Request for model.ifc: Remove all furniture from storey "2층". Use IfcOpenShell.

First a look at what the model holds.

```python
import ifcopenshell
import ifcopenshell.util.element

model = ifcopenshell.open("model.ifc")
print(model.schema)
storey = next(s for s in model.by_type("IfcBuildingStorey") if s.Name == "2층")
furniture = [e for e in ifcopenshell.util.element.get_decomposition(storey) if e.is_a("IfcFurnishingElement")]
seen = {}
for e in furniture:
    element_type = ifcopenshell.util.element.get_type(e)
    name = element_type.Name if element_type not in (None, e) else None
    seen[name] = seen.get(name, 0) + 1
for name, count in sorted(seen.items(), key=str):
    print(count, "x", name)
```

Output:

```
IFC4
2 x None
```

```python
import ifcopenshell
import ifcopenshell.api.root
import ifcopenshell.util.element

model = ifcopenshell.open("model.ifc")

storey = next(s for s in model.by_type("IfcBuildingStorey") if s.Name == "2층")
furniture = [e for e in ifcopenshell.util.element.get_decomposition(storey) if e.is_a("IfcFurnishingElement")]

for e in furniture:
    ifcopenshell.api.root.remove_product(model, product=e)
print(len(furniture), "removed")

model.write("model_v2.ifc")
```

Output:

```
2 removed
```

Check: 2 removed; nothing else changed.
